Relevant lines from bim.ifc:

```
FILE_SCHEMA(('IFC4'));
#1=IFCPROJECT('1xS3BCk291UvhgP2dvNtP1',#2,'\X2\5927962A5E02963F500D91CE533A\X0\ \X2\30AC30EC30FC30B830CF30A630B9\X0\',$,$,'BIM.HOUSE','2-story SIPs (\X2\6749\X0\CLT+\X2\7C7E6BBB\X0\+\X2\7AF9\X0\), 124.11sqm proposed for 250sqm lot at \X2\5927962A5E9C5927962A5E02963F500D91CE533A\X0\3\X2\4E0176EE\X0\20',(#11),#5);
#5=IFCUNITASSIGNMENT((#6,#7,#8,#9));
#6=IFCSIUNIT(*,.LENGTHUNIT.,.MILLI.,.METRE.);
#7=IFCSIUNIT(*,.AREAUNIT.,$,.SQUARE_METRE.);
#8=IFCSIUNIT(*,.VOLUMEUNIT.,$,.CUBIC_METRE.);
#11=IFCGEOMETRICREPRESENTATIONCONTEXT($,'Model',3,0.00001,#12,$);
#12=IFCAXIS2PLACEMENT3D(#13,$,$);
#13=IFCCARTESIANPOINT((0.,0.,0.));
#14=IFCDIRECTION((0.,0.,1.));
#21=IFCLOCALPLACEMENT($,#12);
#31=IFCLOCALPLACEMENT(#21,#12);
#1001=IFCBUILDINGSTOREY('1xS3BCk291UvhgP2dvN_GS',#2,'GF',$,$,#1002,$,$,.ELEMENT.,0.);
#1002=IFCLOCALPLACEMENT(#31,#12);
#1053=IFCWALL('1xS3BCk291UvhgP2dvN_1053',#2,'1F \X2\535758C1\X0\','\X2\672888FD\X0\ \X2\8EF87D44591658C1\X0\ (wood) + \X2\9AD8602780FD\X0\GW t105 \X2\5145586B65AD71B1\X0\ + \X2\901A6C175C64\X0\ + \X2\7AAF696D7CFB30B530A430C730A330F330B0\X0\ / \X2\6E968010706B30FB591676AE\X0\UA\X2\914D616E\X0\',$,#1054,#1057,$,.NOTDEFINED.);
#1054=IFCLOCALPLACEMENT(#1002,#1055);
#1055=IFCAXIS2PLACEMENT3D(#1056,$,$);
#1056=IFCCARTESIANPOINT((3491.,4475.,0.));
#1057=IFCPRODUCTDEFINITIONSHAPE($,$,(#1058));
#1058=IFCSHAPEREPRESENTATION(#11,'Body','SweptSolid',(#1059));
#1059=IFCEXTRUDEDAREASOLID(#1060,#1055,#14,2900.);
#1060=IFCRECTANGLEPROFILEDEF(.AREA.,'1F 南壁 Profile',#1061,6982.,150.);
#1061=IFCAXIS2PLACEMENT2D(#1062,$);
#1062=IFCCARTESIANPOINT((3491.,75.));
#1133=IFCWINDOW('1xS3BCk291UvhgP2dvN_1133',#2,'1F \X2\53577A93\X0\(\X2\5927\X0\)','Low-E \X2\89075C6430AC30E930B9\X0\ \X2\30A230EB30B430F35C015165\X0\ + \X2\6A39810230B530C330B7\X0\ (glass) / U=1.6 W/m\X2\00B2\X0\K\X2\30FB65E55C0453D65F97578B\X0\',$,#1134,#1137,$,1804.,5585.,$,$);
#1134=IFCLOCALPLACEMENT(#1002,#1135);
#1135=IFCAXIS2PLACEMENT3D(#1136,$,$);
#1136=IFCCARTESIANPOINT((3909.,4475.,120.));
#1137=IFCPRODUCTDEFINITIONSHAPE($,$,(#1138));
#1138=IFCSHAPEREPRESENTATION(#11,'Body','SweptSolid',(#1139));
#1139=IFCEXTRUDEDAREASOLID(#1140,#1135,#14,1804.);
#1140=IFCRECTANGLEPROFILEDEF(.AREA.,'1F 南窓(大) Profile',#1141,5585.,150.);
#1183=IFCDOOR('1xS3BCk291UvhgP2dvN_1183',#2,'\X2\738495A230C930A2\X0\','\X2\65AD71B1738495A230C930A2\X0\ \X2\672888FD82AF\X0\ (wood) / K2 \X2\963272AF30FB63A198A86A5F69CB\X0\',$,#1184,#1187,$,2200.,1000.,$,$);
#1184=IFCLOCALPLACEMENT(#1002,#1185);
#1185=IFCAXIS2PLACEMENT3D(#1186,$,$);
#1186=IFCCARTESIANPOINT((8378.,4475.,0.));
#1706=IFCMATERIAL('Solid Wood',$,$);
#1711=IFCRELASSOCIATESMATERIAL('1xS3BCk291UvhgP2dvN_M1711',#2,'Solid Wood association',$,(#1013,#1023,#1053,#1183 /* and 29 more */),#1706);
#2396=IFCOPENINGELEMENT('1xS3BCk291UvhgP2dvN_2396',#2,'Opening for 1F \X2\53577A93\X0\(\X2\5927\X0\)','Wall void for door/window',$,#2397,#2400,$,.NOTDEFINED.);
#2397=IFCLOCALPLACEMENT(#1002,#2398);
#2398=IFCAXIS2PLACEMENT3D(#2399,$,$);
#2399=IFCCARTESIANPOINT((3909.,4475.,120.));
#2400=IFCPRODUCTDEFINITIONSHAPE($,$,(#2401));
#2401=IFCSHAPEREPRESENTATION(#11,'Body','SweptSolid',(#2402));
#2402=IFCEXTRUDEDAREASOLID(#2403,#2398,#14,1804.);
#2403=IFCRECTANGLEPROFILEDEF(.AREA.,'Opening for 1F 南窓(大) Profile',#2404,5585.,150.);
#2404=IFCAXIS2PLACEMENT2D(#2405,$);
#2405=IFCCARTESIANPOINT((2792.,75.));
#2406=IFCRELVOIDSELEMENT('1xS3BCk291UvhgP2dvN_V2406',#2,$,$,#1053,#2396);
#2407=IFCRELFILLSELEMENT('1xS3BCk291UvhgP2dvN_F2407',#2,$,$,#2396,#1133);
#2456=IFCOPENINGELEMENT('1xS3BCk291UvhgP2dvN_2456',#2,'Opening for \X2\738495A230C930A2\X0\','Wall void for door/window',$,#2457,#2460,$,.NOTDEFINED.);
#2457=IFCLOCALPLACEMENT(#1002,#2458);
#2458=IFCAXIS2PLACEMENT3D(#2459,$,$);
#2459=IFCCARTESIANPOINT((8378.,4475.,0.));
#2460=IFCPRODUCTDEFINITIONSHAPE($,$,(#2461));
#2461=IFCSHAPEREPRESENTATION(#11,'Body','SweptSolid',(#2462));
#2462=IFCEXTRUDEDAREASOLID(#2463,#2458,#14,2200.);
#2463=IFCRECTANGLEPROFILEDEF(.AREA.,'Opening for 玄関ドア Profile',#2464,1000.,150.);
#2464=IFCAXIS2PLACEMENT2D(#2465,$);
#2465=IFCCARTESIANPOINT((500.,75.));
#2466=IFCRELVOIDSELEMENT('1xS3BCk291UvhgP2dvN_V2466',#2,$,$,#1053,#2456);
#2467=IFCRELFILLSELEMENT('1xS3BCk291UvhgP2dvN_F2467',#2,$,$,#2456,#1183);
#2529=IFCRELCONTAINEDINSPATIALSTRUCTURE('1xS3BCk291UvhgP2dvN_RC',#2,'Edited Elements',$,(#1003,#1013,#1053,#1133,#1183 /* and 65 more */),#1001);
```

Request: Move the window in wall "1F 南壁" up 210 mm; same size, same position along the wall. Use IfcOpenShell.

```python
import numpy as np
import ifcopenshell
import ifcopenshell.api.geometry
import ifcopenshell.util.placement
import ifcopenshell.util.unit

model = ifcopenshell.open("bim.ifc")
unit_scale = ifcopenshell.util.unit.calculate_unit_scale(model)

window = model.by_guid("1xS3BCk291UvhgP2dvN_1133")
opening = window.FillsVoids[0].RelatingOpeningElement
dz = 210.0

shift = np.array([0.0, 0.0, dz])
# The window is not placed relative to its opening, so move both.
for product in (opening, window):
    matrix = ifcopenshell.util.placement.get_local_placement(product.ObjectPlacement)
    matrix[:3, 3] += shift
    ifcopenshell.api.geometry.edit_object_placement(model, product=product, matrix=matrix, is_si=False)

print(f"moved by {dz * unit_scale:+.3f} m")

model.write("bim_updated.ifc")
```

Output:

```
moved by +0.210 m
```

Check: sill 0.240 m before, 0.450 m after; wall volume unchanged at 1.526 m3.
